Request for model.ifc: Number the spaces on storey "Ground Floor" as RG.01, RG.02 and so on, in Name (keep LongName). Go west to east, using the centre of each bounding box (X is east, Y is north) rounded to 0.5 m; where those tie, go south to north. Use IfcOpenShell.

First a look at what the model holds.

```python
import ifcopenshell
import ifcopenshell.util.element
import ifcopenshell.util.placement

model = ifcopenshell.open("model.ifc")
print(model.schema)
storey = next(s for s in model.by_type("IfcBuildingStorey") if s.Name == "Ground Floor")
spaces = [e for e in ifcopenshell.util.element.get_decomposition(storey) if e.is_a("IfcSpace")]
for e in sorted(spaces, key=lambda e: e.id()):
    origin = ifcopenshell.util.placement.get_local_placement(e.ObjectPlacement)[:3, 3]
    print(e.id(), e.Name, e.LongName, origin.round(2) + 0.0, sep=" | ")
```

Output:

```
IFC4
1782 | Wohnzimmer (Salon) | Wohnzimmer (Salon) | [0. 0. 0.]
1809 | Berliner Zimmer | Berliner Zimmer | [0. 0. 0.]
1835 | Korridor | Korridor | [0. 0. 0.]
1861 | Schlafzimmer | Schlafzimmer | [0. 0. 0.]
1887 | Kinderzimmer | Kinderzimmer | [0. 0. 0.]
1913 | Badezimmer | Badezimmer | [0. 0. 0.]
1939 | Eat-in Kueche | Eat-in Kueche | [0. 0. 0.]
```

```python
import ifcopenshell
import ifcopenshell.geom
import ifcopenshell.util.element
import ifcopenshell.util.shape

model = ifcopenshell.open("model.ifc")
settings = ifcopenshell.geom.settings()
settings.set("use-world-coords", True)


def centre(element):
    shape = ifcopenshell.geom.create_shape(settings, element)
    return ifcopenshell.util.shape.get_bbox_centroid(shape.geometry)


storey = next(s for s in model.by_type("IfcBuildingStorey") if s.Name == "Ground Floor")
spaces = [e for e in ifcopenshell.util.element.get_decomposition(storey) if e.is_a("IfcSpace")]

# Insertion points can sit at a corner or the storey origin, so sort by the geometry (in metres).
centres = {e: centre(e) for e in spaces}
spaces.sort(key=lambda e: (round(centres[e][0] / 0.5), centres[e][1]))

for i, e in enumerate(spaces, start=1):
    number = f"RG.{i:02d}"
    e.Name = number
    print(e.id(), number)

model.write("model_v2.ifc")
```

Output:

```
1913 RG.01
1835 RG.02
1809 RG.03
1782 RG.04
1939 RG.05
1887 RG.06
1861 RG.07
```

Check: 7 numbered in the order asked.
